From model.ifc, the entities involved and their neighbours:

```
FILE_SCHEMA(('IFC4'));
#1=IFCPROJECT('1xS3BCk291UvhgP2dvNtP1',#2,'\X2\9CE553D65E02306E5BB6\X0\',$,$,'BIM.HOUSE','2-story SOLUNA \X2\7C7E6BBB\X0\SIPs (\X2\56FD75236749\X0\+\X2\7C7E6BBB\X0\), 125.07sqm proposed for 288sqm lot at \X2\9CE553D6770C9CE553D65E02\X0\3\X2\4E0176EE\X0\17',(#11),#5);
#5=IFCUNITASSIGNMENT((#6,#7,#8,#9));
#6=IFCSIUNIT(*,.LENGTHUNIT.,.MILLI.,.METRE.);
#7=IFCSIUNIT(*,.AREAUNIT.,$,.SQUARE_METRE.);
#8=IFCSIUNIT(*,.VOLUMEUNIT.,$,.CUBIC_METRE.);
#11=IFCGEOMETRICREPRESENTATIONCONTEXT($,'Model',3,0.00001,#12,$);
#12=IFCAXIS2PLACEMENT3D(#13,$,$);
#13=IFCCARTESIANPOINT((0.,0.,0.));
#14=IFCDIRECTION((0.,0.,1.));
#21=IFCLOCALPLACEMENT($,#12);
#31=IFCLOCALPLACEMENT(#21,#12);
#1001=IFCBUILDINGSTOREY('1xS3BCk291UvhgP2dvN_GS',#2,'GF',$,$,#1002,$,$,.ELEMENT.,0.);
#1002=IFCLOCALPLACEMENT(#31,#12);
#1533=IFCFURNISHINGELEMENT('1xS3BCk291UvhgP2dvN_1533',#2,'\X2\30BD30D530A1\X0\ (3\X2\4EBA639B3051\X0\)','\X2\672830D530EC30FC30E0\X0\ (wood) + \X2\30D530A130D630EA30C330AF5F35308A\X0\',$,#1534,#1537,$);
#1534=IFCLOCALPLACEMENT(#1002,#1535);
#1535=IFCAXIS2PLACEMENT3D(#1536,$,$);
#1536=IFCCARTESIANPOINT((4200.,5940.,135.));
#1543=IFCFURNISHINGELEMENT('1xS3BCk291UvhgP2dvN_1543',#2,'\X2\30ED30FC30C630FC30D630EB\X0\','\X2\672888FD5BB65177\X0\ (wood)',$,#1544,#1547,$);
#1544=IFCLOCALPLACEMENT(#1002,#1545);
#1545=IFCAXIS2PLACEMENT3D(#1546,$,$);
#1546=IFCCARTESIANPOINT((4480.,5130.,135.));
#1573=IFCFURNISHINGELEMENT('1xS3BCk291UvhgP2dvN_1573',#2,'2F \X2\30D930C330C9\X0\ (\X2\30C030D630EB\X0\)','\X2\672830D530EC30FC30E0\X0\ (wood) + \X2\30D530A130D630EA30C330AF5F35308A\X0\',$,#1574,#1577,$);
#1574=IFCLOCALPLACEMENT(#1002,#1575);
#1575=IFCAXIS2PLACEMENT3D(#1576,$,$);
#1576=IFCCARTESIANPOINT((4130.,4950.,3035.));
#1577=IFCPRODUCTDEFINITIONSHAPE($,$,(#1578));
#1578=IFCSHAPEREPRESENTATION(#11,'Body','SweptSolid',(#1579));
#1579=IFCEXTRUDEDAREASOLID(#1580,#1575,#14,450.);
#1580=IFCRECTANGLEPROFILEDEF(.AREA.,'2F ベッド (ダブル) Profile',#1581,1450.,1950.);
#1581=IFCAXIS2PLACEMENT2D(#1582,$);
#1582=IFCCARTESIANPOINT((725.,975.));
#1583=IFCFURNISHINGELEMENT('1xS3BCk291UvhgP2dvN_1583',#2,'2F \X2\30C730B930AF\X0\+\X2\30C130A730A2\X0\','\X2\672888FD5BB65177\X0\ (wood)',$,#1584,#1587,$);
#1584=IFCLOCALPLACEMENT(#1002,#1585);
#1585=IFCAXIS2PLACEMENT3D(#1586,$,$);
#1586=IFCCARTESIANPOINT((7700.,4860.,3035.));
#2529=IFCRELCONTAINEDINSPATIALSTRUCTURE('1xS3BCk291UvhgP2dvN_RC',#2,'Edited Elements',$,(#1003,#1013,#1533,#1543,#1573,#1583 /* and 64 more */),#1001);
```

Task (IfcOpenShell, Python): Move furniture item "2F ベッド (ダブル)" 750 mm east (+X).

```python
import ifcopenshell
import ifcopenshell.api.geometry
import ifcopenshell.util.placement

model = ifcopenshell.open("model.ifc")

item = model.by_guid("1xS3BCk291UvhgP2dvN_1573")
matrix = ifcopenshell.util.placement.get_local_placement(item.ObjectPlacement)
matrix[0, 3] += 750.0
ifcopenshell.api.geometry.edit_object_placement(model, product=item, matrix=matrix, is_si=False)

print(ifcopenshell.util.placement.get_local_placement(item.ObjectPlacement).round(3) + 0.0)

model.write("model-out.ifc")
```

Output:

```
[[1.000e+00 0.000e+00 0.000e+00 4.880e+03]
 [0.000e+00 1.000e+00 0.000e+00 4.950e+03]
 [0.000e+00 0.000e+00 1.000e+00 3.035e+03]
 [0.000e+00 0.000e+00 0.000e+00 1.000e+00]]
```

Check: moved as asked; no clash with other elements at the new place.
